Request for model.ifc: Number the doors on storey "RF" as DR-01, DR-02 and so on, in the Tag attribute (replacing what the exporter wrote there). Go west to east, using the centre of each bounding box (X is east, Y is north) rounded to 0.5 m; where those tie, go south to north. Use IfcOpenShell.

First a look at what the model holds.

```python
import ifcopenshell
import ifcopenshell.util.element
import ifcopenshell.util.placement

model = ifcopenshell.open("model.ifc")
print(model.schema)
storey = next(s for s in model.by_type("IfcBuildingStorey") if s.Name == "RF")
doors = [e for e in ifcopenshell.util.element.get_decomposition(storey) if e.is_a("IfcDoor")]
for e in sorted(doors, key=lambda e: e.id()):
    origin = ifcopenshell.util.placement.get_local_placement(e.ObjectPlacement)[:3, 3]
    print(e.id(), e.Tag, e.Name, origin.round(2) + 0.0, sep=" | ")
```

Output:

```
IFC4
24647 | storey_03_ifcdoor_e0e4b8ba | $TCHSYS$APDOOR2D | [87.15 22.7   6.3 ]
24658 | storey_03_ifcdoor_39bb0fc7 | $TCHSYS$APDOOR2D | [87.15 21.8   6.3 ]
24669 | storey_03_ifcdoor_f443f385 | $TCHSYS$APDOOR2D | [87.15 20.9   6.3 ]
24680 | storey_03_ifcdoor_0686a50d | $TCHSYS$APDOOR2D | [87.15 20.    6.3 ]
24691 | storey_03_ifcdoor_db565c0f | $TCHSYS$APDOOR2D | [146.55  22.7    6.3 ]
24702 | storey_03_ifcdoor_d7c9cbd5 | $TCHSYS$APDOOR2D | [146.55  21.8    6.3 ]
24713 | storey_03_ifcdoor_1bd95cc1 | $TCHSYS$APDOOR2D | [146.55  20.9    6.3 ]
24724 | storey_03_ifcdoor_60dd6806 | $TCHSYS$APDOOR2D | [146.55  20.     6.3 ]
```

```python
import ifcopenshell
import ifcopenshell.geom
import ifcopenshell.util.element
import ifcopenshell.util.shape

model = ifcopenshell.open("model.ifc")
settings = ifcopenshell.geom.settings()
settings.set("use-world-coords", True)


def centre(element):
    shape = ifcopenshell.geom.create_shape(settings, element)
    return ifcopenshell.util.shape.get_bbox_centroid(shape.geometry)


storey = next(s for s in model.by_type("IfcBuildingStorey") if s.Name == "RF")
doors = [e for e in ifcopenshell.util.element.get_decomposition(storey) if e.is_a("IfcDoor")]

# Insertion points can sit at a corner or the storey origin, so sort by the geometry (in metres).
centres = {e: centre(e) for e in doors}
doors.sort(key=lambda e: (round(centres[e][0] / 0.5), centres[e][1]))

for i, e in enumerate(doors, start=1):
    number = f"DR-{i:02d}"
    e.Tag = number
    print(e.id(), number)

model.write("model_edited.ifc")
```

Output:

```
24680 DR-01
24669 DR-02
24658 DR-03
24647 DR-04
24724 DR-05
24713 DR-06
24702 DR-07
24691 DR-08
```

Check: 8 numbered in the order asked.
